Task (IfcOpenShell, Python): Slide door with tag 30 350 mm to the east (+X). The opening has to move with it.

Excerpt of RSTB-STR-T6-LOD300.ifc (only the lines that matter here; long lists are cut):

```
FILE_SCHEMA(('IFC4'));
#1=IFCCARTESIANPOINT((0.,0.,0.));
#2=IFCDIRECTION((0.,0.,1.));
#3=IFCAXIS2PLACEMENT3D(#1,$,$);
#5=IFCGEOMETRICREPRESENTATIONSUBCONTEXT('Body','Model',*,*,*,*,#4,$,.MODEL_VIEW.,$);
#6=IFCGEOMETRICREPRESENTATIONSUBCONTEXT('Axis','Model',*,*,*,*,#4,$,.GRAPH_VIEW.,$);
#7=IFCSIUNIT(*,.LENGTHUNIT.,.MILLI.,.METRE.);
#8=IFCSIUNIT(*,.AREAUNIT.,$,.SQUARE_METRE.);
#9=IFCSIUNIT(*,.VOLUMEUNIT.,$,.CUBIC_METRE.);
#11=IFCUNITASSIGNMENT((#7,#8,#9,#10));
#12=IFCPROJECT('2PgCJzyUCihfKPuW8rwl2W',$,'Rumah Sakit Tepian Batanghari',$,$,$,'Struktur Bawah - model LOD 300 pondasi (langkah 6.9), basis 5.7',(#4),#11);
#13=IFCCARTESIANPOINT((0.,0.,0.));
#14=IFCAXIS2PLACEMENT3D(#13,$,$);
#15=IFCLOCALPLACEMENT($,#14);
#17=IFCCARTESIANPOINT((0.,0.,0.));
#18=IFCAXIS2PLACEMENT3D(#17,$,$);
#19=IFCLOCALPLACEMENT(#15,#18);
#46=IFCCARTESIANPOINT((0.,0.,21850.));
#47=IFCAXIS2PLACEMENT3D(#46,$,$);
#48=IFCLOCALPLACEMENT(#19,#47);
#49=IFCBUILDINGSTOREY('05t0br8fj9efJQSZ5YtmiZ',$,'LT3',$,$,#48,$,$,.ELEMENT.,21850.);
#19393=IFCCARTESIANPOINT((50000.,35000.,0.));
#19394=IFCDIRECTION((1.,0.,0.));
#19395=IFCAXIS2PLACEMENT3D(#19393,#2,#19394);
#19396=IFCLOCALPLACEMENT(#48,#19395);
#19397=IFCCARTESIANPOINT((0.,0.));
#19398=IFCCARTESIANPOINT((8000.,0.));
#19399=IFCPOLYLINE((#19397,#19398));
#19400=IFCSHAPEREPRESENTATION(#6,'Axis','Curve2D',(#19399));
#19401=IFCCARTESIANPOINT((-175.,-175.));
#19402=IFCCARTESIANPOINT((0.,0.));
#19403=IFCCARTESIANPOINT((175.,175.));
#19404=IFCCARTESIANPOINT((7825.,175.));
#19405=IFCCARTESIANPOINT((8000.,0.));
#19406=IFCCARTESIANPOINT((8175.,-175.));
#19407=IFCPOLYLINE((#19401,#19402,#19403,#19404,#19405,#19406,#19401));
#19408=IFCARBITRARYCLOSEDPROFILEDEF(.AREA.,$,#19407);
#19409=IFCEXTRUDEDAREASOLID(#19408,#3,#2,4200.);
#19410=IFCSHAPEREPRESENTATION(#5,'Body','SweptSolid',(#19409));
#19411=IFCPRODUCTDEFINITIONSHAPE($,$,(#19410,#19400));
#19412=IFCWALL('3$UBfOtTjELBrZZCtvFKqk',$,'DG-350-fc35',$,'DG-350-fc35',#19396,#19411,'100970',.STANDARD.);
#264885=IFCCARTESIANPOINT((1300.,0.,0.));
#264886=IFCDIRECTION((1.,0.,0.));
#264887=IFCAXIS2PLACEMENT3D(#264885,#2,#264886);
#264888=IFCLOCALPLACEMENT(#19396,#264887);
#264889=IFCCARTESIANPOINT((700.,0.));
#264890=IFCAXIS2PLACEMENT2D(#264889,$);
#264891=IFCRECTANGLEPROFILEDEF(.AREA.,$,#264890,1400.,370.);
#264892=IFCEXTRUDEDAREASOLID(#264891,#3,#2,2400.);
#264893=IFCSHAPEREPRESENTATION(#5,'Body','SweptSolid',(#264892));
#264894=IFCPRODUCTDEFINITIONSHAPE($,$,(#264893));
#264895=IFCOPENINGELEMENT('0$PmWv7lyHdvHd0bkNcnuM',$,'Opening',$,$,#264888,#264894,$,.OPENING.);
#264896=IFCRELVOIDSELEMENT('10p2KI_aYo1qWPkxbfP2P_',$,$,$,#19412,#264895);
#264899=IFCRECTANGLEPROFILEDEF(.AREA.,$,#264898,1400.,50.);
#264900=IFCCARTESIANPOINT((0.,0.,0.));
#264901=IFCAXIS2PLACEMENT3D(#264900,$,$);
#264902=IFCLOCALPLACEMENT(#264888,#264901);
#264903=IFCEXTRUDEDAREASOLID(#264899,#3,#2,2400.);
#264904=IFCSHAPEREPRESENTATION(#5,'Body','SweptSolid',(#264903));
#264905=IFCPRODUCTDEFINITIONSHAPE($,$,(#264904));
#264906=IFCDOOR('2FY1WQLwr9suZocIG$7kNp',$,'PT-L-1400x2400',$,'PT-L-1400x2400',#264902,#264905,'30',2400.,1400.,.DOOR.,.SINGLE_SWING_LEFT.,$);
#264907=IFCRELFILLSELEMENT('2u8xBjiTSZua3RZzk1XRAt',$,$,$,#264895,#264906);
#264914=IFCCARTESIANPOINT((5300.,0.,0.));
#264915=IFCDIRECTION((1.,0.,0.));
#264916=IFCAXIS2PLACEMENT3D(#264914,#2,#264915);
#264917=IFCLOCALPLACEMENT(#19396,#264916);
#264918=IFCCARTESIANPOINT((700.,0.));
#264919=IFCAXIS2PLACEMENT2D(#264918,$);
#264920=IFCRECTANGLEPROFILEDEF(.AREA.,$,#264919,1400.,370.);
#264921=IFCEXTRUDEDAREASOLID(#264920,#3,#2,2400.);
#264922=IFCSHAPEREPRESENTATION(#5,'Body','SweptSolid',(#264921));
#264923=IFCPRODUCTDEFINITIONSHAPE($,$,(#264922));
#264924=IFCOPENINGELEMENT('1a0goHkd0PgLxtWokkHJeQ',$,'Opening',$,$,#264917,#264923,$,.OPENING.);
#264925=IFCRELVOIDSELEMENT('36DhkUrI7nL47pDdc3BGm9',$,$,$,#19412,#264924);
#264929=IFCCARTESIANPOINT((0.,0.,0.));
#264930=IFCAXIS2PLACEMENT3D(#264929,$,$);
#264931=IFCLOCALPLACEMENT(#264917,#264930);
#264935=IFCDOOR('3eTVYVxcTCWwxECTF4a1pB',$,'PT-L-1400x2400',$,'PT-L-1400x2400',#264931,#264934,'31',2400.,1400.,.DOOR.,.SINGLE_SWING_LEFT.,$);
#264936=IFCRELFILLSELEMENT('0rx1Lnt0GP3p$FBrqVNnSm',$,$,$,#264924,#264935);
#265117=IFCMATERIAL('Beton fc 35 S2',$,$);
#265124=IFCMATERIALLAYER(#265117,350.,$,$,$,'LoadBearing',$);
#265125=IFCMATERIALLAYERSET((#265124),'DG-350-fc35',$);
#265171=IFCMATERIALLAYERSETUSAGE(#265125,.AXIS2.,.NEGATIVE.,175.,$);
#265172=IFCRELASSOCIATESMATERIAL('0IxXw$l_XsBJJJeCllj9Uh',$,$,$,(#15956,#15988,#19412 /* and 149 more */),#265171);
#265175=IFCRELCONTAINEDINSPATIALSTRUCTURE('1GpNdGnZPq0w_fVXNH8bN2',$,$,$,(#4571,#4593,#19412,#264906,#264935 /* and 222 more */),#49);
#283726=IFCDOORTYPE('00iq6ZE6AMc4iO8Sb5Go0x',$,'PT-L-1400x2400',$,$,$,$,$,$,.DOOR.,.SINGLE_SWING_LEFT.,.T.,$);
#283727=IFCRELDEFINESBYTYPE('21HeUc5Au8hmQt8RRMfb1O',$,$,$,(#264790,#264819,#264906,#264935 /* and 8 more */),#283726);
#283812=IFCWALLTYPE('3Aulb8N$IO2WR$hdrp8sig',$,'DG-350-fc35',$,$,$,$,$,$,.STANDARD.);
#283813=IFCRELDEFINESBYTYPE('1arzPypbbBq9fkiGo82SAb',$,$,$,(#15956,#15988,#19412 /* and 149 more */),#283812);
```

```python
import ifcopenshell
import ifcopenshell.api.geometry
import ifcopenshell.util.placement
import ifcopenshell.util.unit

model = ifcopenshell.open("RSTB-STR-T6-LOD300.ifc")
unit_scale = ifcopenshell.util.unit.calculate_unit_scale(model)

door = model.by_guid("2FY1WQLwr9suZocIG$7kNp")
opening = door.FillsVoids[0].RelatingOpeningElement
wall = opening.VoidsElements[0].RelatingBuildingElement

wall_matrix = ifcopenshell.util.placement.get_local_placement(wall.ObjectPlacement)
shift = wall_matrix[:3, 0] * 0.35 / unit_scale
before = ifcopenshell.util.placement.get_local_placement(door.ObjectPlacement)[:3, 3].copy()

# The door is placed relative to its opening, so it follows when the opening moves.
matrix = ifcopenshell.util.placement.get_local_placement(opening.ObjectPlacement)
matrix[:3, 3] += shift
ifcopenshell.api.geometry.edit_object_placement(
    model, product=opening, matrix=matrix, is_si=False, should_transform_children=True
)

after = ifcopenshell.util.placement.get_local_placement(door.ObjectPlacement)[:3, 3]
print("door moved by", (after - before).round(3) + 0.0)

model.write("RSTB-STR-T6-LOD300_edited.ifc")
```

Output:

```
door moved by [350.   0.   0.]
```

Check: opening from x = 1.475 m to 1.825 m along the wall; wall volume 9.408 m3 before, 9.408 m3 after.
